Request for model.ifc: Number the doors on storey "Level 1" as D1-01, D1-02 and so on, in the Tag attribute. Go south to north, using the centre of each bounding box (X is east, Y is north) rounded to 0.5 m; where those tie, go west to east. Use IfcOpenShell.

First a look at what the model holds.

```python
import ifcopenshell
import ifcopenshell.util.element
import ifcopenshell.util.placement

model = ifcopenshell.open("model.ifc")
print(model.schema)
storey = next(s for s in model.by_type("IfcBuildingStorey") if s.Name == "Level 1")
doors = [e for e in ifcopenshell.util.element.get_decomposition(storey) if e.is_a("IfcDoor")]
for e in sorted(doors, key=lambda e: e.id()):
    origin = ifcopenshell.util.placement.get_local_placement(e.ObjectPlacement)[:3, 3]
    print(e.id(), e.Tag, e.Name, origin.round(2) + 0.0, sep=" | ")
```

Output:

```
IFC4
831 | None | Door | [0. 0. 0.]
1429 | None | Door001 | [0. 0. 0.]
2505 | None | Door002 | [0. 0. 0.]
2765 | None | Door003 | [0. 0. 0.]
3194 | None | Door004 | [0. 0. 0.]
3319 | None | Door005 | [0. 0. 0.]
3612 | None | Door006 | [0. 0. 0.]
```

```python
import ifcopenshell
import ifcopenshell.geom
import ifcopenshell.util.element
import ifcopenshell.util.shape

model = ifcopenshell.open("model.ifc")
settings = ifcopenshell.geom.settings()
settings.set("use-world-coords", True)


def centre(element):
    shape = ifcopenshell.geom.create_shape(settings, element)
    return ifcopenshell.util.shape.get_bbox_centroid(shape.geometry)


storey = next(s for s in model.by_type("IfcBuildingStorey") if s.Name == "Level 1")
doors = [e for e in ifcopenshell.util.element.get_decomposition(storey) if e.is_a("IfcDoor")]

# Insertion points can sit at a corner or the storey origin, so sort by the geometry (in metres).
centres = {e: centre(e) for e in doors}
doors.sort(key=lambda e: (round(centres[e][1] / 0.5), centres[e][0]))

for i, e in enumerate(doors, start=1):
    number = f"D1-{i:02d}"
    e.Tag = number
    print(e.id(), number)

model.write("model-out.ifc")
```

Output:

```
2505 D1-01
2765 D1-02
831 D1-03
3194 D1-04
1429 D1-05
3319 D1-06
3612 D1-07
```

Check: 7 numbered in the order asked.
